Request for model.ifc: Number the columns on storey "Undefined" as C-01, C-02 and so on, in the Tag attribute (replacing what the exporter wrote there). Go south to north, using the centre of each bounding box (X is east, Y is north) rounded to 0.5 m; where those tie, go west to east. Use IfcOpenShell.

First a look at what the model holds.

```python
import ifcopenshell
import ifcopenshell.util.element
import ifcopenshell.util.placement

model = ifcopenshell.open("model.ifc")
print(model.schema)
storey = next(s for s in model.by_type("IfcBuildingStorey") if s.Name == "Undefined")
columns = [e for e in ifcopenshell.util.element.get_decomposition(storey) if e.is_a("IfcColumn")]
for e in sorted(columns, key=lambda e: e.id()):
    origin = ifcopenshell.util.placement.get_local_placement(e.ObjectPlacement)[:3, 3]
    print(e.id(), e.Tag, e.Name, origin.round(2) + 0.0, sep=" | ")
```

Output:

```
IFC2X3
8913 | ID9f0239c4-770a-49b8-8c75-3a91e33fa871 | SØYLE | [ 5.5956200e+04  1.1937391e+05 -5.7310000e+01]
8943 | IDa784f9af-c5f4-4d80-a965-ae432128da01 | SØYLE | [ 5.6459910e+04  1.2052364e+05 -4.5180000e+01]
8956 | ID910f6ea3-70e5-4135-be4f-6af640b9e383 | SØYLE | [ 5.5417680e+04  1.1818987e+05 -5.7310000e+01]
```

```python
import ifcopenshell
import ifcopenshell.geom
import ifcopenshell.util.element
import ifcopenshell.util.shape

model = ifcopenshell.open("model.ifc")
settings = ifcopenshell.geom.settings()
settings.set("use-world-coords", True)


def centre(element):
    shape = ifcopenshell.geom.create_shape(settings, element)
    return ifcopenshell.util.shape.get_bbox_centroid(shape.geometry)


storey = next(s for s in model.by_type("IfcBuildingStorey") if s.Name == "Undefined")
columns = [e for e in ifcopenshell.util.element.get_decomposition(storey) if e.is_a("IfcColumn")]

# Insertion points can sit at a corner or the storey origin, so sort by the geometry (in metres).
centres = {e: centre(e) for e in columns}
columns.sort(key=lambda e: (round(centres[e][1] / 0.5), centres[e][0]))

for i, e in enumerate(columns, start=1):
    number = f"C-{i:02d}"
    e.Tag = number
    print(e.id(), number)

model.write("model-out.ifc")
```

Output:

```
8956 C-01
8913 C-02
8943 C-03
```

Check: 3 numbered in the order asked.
